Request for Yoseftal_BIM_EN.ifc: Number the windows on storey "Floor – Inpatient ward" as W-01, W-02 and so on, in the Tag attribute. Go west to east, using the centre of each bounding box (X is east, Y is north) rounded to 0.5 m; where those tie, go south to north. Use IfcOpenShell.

First a look at what the model holds.

```python
import ifcopenshell
import ifcopenshell.util.element
import ifcopenshell.util.placement

model = ifcopenshell.open("Yoseftal_BIM_EN.ifc")
print(model.schema)
storey = next(s for s in model.by_type("IfcBuildingStorey") if s.Name == "Floor – Inpatient ward")
windows = [e for e in ifcopenshell.util.element.get_decomposition(storey) if e.is_a("IfcWindow")]
for e in sorted(windows, key=lambda e: e.id()):
    origin = ifcopenshell.util.placement.get_local_placement(e.ObjectPlacement)[:3, 3]
    print(e.id(), e.Tag, e.Name, origin.round(2) + 0.0, sep=" | ")
```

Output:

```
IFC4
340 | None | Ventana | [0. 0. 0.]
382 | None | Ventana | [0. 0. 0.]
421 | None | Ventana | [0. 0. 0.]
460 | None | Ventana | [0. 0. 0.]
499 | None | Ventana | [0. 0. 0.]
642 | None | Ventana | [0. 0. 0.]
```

```python
import ifcopenshell
import ifcopenshell.geom
import ifcopenshell.util.element
import ifcopenshell.util.shape

model = ifcopenshell.open("Yoseftal_BIM_EN.ifc")
settings = ifcopenshell.geom.settings()
settings.set("use-world-coords", True)


def centre(element):
    shape = ifcopenshell.geom.create_shape(settings, element)
    return ifcopenshell.util.shape.get_bbox_centroid(shape.geometry)


storey = next(s for s in model.by_type("IfcBuildingStorey") if s.Name == "Floor – Inpatient ward")
windows = [e for e in ifcopenshell.util.element.get_decomposition(storey) if e.is_a("IfcWindow")]

# Insertion points can sit at a corner or the storey origin, so sort by the geometry (in metres).
centres = {e: centre(e) for e in windows}
windows.sort(key=lambda e: (round(centres[e][0] / 0.5), centres[e][1]))

for i, e in enumerate(windows, start=1):
    number = f"W-{i:02d}"
    e.Tag = number
    print(e.id(), number)

model.write("Yoseftal_BIM_EN-out.ifc")
```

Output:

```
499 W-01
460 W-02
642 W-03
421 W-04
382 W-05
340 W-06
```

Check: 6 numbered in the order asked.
